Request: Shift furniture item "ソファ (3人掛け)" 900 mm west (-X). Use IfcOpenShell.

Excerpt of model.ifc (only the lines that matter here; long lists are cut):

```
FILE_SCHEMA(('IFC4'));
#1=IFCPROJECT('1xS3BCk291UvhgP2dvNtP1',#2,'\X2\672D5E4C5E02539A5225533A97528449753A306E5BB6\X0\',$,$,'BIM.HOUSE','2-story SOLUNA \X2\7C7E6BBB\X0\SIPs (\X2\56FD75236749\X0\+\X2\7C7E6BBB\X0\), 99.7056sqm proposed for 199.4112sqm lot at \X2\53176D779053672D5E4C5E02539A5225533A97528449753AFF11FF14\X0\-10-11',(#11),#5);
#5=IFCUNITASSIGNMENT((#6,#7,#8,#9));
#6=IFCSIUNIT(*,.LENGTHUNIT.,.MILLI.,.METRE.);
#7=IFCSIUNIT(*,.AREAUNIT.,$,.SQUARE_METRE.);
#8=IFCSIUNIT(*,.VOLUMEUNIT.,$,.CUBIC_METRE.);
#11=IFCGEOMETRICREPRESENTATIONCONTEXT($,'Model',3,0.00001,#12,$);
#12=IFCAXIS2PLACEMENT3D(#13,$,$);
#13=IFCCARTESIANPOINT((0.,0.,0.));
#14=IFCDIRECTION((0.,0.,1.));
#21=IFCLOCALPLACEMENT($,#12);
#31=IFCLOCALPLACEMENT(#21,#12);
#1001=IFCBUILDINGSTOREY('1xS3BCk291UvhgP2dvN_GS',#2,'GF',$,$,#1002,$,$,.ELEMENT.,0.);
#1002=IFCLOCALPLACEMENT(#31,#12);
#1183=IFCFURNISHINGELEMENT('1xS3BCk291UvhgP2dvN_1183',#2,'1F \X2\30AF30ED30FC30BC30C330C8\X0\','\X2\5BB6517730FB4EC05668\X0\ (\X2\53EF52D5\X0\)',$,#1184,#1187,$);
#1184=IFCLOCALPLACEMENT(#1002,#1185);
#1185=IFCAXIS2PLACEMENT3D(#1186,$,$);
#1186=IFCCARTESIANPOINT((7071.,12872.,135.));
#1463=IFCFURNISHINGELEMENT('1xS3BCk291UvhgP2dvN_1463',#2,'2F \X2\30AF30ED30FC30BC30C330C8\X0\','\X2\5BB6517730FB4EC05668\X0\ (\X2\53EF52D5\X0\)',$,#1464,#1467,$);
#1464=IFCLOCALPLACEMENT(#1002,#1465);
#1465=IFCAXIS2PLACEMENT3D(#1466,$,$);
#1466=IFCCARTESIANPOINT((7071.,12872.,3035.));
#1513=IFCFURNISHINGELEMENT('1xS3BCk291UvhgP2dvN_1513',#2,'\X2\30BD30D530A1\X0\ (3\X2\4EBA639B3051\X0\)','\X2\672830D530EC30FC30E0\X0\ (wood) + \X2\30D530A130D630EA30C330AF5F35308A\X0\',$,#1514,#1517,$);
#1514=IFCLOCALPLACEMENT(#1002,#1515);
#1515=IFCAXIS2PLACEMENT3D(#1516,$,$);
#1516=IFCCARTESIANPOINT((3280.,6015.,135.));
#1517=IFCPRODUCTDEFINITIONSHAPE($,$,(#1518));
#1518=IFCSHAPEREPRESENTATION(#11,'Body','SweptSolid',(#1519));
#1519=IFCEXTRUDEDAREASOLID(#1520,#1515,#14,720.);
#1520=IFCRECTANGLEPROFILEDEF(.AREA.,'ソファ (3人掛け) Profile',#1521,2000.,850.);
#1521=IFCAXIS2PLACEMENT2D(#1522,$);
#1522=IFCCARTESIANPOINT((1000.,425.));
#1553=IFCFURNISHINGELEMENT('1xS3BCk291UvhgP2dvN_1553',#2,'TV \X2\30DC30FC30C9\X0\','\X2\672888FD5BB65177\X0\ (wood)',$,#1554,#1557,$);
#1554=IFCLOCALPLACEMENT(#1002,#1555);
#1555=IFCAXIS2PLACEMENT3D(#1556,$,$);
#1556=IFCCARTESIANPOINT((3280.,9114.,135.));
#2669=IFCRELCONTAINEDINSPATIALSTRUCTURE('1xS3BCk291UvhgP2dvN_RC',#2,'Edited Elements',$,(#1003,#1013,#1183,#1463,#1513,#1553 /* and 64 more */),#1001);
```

```python
import ifcopenshell
import ifcopenshell.api.geometry
import ifcopenshell.util.placement

model = ifcopenshell.open("model.ifc")

item = model.by_guid("1xS3BCk291UvhgP2dvN_1513")
matrix = ifcopenshell.util.placement.get_local_placement(item.ObjectPlacement)
matrix[0, 3] -= 900.0
ifcopenshell.api.geometry.edit_object_placement(model, product=item, matrix=matrix, is_si=False)

print(ifcopenshell.util.placement.get_local_placement(item.ObjectPlacement).round(3) + 0.0)

model.write("model_rev.ifc")
```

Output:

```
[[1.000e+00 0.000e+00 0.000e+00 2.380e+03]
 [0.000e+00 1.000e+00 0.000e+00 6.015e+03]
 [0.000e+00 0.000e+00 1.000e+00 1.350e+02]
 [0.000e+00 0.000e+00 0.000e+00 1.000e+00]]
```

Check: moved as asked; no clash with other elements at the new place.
